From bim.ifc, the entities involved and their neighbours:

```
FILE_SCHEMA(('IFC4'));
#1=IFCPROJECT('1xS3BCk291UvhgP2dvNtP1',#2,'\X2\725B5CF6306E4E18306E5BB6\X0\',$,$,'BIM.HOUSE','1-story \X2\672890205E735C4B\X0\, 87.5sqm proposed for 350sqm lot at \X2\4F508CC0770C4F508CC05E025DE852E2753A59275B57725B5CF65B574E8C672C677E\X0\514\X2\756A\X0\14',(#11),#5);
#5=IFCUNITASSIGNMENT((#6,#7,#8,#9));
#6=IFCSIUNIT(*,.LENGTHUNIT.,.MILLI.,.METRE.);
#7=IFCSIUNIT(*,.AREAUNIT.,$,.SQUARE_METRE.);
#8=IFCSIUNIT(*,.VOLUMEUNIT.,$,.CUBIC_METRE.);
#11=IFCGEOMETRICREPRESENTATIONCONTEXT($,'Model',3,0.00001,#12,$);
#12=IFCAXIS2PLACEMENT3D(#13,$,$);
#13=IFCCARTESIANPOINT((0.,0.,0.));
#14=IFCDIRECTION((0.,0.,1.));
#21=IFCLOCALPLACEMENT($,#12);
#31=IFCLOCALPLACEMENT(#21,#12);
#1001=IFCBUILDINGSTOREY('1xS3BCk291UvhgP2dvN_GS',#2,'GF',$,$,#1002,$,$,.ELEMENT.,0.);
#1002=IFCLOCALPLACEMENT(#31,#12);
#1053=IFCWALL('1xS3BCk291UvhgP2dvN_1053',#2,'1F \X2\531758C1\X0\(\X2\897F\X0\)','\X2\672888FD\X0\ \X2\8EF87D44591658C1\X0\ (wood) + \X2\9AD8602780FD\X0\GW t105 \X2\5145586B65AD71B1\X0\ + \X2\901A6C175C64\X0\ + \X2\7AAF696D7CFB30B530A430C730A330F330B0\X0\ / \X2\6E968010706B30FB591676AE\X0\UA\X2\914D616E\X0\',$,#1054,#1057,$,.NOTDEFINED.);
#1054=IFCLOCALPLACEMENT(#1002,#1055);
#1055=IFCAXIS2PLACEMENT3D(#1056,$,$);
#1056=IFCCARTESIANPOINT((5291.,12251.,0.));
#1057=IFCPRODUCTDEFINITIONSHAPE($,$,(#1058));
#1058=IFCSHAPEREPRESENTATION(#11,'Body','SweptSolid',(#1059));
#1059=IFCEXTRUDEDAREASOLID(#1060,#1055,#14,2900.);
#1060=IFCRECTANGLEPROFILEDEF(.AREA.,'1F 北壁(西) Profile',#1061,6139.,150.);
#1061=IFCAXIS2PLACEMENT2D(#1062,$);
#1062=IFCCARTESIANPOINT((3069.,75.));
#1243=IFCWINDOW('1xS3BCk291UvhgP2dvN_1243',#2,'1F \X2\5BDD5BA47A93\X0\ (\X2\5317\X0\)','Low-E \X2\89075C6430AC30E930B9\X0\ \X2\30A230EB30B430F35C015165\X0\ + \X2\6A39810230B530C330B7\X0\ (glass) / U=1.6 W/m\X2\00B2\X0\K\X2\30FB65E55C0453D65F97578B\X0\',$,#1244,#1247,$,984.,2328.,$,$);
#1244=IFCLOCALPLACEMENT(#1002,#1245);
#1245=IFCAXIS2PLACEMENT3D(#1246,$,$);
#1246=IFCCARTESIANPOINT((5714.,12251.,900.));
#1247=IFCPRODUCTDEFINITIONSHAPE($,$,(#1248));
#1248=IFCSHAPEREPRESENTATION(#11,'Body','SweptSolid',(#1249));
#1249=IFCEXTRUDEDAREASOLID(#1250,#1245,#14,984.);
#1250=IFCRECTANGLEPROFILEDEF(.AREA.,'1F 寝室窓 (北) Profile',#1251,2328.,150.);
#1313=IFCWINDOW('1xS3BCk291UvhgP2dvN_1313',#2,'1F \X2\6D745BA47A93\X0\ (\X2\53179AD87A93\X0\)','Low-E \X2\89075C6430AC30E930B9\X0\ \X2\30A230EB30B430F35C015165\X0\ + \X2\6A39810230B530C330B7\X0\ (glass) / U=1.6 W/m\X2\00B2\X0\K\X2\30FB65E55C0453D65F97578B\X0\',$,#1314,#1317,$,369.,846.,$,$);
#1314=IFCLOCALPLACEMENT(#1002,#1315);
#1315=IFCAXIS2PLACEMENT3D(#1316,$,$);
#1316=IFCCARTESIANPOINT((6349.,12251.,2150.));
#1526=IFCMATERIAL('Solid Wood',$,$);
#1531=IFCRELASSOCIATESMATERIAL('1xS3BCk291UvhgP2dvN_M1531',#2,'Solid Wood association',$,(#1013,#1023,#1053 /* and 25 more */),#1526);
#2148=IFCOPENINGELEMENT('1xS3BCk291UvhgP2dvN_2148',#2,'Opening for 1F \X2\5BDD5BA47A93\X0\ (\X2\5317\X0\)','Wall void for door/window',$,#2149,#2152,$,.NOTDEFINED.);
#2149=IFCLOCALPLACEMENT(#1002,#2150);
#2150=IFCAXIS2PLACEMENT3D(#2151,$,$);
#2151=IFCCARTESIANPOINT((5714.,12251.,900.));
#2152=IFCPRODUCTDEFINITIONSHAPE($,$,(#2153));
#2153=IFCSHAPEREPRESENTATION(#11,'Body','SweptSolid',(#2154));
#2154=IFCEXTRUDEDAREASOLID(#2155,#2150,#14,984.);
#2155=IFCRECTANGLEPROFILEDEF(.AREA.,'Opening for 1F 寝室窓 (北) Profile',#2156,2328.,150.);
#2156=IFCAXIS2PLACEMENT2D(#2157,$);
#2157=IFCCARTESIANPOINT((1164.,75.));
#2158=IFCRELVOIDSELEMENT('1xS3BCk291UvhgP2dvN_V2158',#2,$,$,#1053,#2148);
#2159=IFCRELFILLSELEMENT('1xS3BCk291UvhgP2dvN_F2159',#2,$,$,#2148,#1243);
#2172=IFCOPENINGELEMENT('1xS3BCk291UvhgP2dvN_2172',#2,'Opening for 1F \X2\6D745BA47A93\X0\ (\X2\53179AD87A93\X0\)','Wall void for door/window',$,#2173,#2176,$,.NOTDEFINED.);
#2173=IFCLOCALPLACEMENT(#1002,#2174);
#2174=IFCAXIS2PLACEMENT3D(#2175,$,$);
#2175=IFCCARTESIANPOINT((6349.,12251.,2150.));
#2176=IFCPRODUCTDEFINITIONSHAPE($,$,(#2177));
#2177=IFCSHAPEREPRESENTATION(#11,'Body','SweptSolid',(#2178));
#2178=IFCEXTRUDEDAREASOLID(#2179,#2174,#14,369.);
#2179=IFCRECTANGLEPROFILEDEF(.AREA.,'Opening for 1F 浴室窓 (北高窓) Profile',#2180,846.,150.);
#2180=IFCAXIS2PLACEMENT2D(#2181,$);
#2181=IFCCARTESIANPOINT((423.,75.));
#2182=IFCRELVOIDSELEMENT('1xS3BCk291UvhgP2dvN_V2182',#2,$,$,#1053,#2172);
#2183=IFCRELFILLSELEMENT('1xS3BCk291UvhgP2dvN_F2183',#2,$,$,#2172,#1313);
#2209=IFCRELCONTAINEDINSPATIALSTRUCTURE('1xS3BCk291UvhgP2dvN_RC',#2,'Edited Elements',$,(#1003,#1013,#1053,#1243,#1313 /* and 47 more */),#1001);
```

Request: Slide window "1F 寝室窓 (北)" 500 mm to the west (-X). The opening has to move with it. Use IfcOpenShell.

```python
import ifcopenshell
import ifcopenshell.api.geometry
import ifcopenshell.util.placement
import ifcopenshell.util.unit

model = ifcopenshell.open("bim.ifc")
unit_scale = ifcopenshell.util.unit.calculate_unit_scale(model)

window = model.by_guid("1xS3BCk291UvhgP2dvN_1243")
opening = window.FillsVoids[0].RelatingOpeningElement
wall = opening.VoidsElements[0].RelatingBuildingElement

wall_matrix = ifcopenshell.util.placement.get_local_placement(wall.ObjectPlacement)
shift = wall_matrix[:3, 0] * -0.5 / unit_scale
before = ifcopenshell.util.placement.get_local_placement(window.ObjectPlacement)[:3, 3].copy()

# The window is not placed relative to its opening, so move both.
for product in (opening, window):
    matrix = ifcopenshell.util.placement.get_local_placement(product.ObjectPlacement)
    matrix[:3, 3] += shift
    ifcopenshell.api.geometry.edit_object_placement(model, product=product, matrix=matrix, is_si=False)

after = ifcopenshell.util.placement.get_local_placement(window.ObjectPlacement)[:3, 3]
print("window moved by", (after - before).round(3) + 0.0)

model.write("bim_updated.ifc")
```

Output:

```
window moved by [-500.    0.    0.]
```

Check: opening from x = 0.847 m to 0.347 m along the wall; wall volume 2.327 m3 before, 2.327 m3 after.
